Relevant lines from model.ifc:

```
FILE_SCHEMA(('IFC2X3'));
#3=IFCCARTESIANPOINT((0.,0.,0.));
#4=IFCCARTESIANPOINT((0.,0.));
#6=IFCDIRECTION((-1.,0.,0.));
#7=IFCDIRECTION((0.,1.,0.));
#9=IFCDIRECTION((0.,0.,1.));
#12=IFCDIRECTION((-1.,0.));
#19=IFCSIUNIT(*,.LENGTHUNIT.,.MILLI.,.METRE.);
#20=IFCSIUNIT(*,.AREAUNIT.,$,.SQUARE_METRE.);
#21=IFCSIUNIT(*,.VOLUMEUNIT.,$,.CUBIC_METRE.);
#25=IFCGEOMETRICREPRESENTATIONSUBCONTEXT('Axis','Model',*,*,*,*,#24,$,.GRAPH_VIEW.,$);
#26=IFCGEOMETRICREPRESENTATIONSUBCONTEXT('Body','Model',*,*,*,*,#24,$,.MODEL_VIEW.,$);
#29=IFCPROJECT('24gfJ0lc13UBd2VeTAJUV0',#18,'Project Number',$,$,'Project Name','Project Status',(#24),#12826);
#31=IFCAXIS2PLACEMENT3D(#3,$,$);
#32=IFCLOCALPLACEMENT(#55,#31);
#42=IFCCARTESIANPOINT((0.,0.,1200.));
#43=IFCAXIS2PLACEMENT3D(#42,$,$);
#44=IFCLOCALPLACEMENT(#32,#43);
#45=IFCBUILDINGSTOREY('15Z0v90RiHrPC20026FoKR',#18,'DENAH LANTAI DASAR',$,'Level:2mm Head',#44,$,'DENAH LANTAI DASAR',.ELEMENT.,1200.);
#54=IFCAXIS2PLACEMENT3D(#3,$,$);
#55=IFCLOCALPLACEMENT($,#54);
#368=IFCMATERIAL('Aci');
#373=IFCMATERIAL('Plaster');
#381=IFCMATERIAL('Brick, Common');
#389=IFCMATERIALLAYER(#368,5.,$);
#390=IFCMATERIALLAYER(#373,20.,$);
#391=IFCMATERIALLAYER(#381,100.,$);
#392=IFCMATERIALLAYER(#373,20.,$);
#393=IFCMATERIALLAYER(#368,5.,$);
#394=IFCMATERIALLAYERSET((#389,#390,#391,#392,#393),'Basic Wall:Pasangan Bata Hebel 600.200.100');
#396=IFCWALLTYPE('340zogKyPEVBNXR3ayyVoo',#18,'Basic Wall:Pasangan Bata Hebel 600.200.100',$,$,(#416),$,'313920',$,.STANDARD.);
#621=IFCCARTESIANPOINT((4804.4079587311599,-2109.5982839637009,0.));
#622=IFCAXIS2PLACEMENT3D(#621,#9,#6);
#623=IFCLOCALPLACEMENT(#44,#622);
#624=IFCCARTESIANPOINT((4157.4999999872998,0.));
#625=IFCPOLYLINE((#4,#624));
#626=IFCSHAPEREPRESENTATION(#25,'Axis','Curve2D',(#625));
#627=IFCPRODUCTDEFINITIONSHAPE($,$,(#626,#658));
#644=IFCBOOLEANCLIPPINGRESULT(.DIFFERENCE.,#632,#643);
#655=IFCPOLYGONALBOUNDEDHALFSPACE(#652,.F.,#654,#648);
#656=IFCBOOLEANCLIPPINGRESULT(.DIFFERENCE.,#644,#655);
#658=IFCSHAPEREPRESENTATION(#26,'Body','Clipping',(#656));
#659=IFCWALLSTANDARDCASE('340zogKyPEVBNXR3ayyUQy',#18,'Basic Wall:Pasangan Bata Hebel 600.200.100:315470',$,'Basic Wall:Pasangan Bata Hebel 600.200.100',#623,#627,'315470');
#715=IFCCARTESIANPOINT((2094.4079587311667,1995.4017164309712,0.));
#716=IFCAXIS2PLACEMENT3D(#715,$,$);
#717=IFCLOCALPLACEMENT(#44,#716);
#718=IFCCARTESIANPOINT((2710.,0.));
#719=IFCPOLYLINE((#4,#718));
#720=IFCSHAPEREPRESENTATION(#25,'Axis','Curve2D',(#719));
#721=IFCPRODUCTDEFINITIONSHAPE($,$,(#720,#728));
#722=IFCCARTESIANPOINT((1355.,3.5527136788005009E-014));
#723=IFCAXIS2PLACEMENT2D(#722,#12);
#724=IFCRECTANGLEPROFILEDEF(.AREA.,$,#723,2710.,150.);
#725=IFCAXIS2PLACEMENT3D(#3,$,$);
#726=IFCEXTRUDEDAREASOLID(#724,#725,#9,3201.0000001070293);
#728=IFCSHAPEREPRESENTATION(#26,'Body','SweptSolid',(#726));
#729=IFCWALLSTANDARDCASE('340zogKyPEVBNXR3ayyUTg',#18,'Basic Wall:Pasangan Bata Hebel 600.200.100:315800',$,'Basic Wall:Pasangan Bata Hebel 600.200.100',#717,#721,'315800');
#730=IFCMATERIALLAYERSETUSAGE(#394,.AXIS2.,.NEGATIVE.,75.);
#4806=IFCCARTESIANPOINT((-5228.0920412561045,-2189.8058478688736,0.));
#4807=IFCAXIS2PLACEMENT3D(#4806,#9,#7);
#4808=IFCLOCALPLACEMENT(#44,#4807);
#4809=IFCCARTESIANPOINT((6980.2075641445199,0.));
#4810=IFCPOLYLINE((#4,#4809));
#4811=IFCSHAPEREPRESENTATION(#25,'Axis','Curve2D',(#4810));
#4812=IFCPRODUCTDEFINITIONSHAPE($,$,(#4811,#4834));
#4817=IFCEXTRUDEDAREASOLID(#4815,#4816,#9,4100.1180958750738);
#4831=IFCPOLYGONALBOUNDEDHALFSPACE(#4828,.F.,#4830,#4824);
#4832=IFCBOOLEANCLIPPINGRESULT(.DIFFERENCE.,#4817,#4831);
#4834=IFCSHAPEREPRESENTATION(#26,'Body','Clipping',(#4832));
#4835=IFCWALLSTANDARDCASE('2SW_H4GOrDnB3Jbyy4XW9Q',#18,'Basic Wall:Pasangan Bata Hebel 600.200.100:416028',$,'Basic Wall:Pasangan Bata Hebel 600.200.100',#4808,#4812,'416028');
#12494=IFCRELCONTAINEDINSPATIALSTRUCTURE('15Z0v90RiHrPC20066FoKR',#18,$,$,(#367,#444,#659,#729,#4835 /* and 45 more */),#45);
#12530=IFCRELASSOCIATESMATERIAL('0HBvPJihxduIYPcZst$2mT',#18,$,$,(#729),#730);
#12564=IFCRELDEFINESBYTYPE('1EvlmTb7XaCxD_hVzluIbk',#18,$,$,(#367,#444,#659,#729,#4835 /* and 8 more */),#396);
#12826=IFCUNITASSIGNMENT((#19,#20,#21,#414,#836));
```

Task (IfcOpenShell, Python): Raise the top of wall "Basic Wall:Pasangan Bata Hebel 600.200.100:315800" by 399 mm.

```python
import ifcopenshell
import ifcopenshell.geom
import ifcopenshell.util.representation
import ifcopenshell.util.shape
import ifcopenshell.util.unit

model = ifcopenshell.open("model.ifc")
unit_scale = ifcopenshell.util.unit.calculate_unit_scale(model)
settings = ifcopenshell.geom.settings()


def volume(element):
    """Net volume in cubic metres, openings subtracted."""
    shape = ifcopenshell.geom.create_shape(settings, element)
    return ifcopenshell.util.shape.get_volume(shape.geometry)


wall = model.by_guid("340zogKyPEVBNXR3ayyUTg")
before = volume(wall)

body = ifcopenshell.util.representation.get_representation(wall, "Model", "Body")
solid = body.Items[0]
old_height = solid.Depth
solid.Depth += 0.399 / unit_scale
after = volume(wall)

print(f"height {old_height:g} -> {solid.Depth:g}, volume {before:.3f} -> {after:.3f} m3")

model.write("model-out.ifc")
```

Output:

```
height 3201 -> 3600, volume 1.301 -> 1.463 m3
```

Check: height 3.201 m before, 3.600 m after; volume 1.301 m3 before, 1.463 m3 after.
